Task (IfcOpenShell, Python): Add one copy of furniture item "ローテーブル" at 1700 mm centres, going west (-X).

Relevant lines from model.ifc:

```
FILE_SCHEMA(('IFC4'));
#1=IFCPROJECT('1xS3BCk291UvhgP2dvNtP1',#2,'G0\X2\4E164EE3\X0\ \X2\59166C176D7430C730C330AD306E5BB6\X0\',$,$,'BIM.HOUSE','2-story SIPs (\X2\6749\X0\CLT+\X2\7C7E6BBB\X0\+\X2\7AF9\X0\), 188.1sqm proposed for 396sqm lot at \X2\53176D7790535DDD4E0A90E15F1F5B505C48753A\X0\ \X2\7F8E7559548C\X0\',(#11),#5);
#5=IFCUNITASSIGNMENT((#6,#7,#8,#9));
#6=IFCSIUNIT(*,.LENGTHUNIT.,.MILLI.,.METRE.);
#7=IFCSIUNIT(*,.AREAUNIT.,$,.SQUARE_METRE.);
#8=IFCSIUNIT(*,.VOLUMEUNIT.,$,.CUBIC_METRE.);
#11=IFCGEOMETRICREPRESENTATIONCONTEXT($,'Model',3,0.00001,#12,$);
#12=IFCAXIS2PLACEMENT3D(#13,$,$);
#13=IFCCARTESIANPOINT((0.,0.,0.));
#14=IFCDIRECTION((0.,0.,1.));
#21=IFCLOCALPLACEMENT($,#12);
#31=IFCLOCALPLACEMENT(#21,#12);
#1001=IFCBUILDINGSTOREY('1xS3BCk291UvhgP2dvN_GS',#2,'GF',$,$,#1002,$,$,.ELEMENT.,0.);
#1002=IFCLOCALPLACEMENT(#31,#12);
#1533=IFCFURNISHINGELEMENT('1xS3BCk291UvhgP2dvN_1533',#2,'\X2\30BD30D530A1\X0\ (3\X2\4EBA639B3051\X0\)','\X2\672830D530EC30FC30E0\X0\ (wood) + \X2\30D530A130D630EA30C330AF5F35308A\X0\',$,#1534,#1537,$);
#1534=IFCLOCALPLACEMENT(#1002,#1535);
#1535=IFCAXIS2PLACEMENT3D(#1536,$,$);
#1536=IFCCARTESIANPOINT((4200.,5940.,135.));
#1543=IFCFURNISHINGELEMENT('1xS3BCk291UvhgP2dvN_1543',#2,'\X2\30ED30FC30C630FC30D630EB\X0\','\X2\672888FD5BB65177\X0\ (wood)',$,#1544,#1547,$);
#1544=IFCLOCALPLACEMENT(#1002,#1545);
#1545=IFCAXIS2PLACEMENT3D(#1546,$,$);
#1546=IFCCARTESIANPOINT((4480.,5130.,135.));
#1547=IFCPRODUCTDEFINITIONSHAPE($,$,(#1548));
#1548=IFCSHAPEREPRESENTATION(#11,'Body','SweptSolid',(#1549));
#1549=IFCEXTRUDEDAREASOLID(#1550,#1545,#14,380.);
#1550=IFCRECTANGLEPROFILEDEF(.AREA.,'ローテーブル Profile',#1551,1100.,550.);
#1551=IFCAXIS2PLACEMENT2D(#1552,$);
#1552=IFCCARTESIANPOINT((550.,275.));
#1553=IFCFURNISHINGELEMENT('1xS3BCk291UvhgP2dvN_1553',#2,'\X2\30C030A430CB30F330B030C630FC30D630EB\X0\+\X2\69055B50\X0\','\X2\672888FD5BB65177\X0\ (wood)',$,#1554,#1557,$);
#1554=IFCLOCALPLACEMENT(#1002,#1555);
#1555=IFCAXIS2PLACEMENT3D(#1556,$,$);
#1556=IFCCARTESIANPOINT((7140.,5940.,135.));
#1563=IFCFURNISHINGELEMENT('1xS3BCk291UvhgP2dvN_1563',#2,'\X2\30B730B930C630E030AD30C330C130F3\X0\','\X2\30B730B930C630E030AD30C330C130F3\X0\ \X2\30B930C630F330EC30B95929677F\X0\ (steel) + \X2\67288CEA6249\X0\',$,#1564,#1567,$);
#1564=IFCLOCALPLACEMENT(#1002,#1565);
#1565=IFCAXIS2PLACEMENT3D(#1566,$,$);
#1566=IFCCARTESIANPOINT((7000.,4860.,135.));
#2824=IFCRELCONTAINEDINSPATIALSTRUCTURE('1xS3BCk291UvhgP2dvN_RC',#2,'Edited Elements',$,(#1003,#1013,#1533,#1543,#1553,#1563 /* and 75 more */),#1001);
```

```python
import numpy as np
import ifcopenshell
import ifcopenshell.api.geometry
import ifcopenshell.api.root
import ifcopenshell.util.element
import ifcopenshell.util.placement
import ifcopenshell.util.unit

model = ifcopenshell.open("model.ifc")
unit_scale = ifcopenshell.util.unit.calculate_unit_scale(model)


def reuse_history(source, copy):
    """copy_class also copies each property set's owner history, people and application; keep the originals."""
    for rel in copy.IsDefinedBy:
        if rel.is_a("IfcRelDefinesByProperties") and (history := rel.RelatingPropertyDefinition.OwnerHistory):
            rel.RelatingPropertyDefinition.OwnerHistory = source.OwnerHistory
            ifcopenshell.util.element.remove_deep2(model, history)


source = model.by_id(1543)
base = ifcopenshell.util.placement.get_local_placement(source.ObjectPlacement)
step = np.array([-1.0, 0.0, 0.0]) * 1.7 / unit_scale

for i in range(1, 2):
    copy = ifcopenshell.api.root.copy_class(model, product=source)
    copy.Representation = ifcopenshell.util.element.copy_deep(
        model, source.Representation, exclude=["IfcGeometricRepresentationContext", "IfcRepresentationMap"]
    )
    reuse_history(source, copy)
    matrix = base.copy()
    matrix[:3, 3] += i * step
    print("added at", matrix[:3, 3].round(3) + 0.0)
    ifcopenshell.api.geometry.edit_object_placement(model, product=copy, matrix=matrix, is_si=False)

model.write("model_v2.ifc")
```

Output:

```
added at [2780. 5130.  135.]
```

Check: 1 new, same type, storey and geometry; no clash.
